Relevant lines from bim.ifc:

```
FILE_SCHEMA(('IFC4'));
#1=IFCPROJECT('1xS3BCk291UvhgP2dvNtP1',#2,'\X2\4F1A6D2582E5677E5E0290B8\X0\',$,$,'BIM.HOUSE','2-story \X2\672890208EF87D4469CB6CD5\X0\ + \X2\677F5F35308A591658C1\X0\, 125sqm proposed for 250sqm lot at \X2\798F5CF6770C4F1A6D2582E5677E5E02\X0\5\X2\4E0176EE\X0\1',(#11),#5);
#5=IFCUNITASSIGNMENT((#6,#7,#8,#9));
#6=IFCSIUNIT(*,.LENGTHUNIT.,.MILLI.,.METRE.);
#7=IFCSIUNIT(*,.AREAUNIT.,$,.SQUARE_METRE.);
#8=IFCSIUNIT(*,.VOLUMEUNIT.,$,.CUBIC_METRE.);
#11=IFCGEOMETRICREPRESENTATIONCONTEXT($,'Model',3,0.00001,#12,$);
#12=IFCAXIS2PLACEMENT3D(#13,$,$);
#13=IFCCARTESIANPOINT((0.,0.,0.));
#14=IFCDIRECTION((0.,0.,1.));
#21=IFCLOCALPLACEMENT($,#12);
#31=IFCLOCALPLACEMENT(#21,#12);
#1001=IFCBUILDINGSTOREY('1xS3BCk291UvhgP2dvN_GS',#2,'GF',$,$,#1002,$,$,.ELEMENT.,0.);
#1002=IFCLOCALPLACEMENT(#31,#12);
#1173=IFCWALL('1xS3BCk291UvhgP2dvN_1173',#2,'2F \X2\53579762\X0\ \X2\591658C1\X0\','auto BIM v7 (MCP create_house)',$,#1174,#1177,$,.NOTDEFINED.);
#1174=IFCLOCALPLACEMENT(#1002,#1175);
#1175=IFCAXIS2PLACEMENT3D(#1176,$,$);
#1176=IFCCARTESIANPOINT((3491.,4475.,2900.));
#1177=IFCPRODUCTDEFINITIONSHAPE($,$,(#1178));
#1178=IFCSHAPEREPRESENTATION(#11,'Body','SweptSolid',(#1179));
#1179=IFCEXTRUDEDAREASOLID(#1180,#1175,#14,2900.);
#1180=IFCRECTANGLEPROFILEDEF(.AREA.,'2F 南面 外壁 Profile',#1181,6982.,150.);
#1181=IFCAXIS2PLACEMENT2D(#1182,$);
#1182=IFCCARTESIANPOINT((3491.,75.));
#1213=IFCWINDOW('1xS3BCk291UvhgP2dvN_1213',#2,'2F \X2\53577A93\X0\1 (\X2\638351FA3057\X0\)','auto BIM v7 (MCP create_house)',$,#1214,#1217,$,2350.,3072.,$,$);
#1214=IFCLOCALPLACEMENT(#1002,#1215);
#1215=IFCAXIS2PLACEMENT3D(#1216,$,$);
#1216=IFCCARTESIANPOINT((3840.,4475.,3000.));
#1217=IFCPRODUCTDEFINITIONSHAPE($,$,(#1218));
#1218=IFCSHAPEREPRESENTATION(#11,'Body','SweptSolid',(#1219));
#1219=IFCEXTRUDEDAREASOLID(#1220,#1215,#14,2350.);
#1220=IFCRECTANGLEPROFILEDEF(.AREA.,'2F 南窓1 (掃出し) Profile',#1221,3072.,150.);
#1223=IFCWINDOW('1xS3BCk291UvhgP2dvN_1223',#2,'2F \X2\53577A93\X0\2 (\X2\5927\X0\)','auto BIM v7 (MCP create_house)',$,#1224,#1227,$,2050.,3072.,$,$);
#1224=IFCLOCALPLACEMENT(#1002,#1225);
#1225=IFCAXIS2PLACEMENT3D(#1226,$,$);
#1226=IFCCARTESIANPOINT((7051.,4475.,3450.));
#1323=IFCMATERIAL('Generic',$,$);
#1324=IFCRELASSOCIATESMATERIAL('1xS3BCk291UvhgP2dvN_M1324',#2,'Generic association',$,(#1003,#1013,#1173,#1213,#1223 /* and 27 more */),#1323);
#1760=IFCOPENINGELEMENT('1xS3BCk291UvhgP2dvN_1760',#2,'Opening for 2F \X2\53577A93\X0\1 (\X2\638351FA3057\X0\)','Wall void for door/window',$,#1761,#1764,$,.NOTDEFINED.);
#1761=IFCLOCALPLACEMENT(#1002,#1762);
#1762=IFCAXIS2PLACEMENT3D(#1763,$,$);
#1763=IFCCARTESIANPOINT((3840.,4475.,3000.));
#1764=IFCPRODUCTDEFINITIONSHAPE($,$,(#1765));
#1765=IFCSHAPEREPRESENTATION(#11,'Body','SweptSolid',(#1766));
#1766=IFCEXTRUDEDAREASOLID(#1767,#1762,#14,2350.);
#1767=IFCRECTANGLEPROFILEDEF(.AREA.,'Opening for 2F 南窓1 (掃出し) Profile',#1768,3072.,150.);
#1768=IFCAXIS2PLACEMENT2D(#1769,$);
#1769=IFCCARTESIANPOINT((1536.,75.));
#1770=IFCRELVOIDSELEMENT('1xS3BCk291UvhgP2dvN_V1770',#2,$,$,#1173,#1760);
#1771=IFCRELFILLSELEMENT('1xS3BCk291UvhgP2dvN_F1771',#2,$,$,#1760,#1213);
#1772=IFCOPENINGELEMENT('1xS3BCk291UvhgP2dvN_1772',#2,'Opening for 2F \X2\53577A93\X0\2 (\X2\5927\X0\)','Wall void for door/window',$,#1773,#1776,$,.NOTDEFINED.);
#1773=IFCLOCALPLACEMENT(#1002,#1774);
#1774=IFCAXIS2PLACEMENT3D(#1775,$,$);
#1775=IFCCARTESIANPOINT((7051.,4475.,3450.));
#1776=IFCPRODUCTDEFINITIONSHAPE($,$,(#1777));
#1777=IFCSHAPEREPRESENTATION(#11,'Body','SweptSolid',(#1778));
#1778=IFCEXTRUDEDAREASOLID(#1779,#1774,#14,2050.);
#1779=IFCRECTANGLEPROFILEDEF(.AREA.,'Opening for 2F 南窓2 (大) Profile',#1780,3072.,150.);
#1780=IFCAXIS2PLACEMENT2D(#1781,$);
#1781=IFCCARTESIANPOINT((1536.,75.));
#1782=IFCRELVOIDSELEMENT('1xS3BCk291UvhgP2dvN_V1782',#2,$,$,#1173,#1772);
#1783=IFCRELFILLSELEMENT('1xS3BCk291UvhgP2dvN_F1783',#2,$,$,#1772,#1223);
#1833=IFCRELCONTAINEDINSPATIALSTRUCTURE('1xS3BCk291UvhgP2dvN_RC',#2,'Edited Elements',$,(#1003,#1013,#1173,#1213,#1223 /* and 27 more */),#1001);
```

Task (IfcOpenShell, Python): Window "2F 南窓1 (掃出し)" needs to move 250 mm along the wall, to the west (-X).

```python
import ifcopenshell
import ifcopenshell.api.geometry
import ifcopenshell.util.placement

model = ifcopenshell.open("bim.ifc")

window = model.by_guid("1xS3BCk291UvhgP2dvN_1213")
opening = window.FillsVoids[0].RelatingOpeningElement
wall = opening.VoidsElements[0].RelatingBuildingElement

wall_matrix = ifcopenshell.util.placement.get_local_placement(wall.ObjectPlacement)
shift = wall_matrix[:3, 0] * -250.0
before = ifcopenshell.util.placement.get_local_placement(window.ObjectPlacement)[:3, 3].copy()

# The window is not placed relative to its opening, so move both.
for product in (opening, window):
    matrix = ifcopenshell.util.placement.get_local_placement(product.ObjectPlacement)
    matrix[:3, 3] += shift
    ifcopenshell.api.geometry.edit_object_placement(model, product=product, matrix=matrix, is_si=False)

after = ifcopenshell.util.placement.get_local_placement(window.ObjectPlacement)[:3, 3]
print("window moved by", (after - before).round(3) + 0.0)

model.write("bim_rev.ifc")
```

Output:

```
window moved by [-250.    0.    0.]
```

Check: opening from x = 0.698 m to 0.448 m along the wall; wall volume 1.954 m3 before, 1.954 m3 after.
